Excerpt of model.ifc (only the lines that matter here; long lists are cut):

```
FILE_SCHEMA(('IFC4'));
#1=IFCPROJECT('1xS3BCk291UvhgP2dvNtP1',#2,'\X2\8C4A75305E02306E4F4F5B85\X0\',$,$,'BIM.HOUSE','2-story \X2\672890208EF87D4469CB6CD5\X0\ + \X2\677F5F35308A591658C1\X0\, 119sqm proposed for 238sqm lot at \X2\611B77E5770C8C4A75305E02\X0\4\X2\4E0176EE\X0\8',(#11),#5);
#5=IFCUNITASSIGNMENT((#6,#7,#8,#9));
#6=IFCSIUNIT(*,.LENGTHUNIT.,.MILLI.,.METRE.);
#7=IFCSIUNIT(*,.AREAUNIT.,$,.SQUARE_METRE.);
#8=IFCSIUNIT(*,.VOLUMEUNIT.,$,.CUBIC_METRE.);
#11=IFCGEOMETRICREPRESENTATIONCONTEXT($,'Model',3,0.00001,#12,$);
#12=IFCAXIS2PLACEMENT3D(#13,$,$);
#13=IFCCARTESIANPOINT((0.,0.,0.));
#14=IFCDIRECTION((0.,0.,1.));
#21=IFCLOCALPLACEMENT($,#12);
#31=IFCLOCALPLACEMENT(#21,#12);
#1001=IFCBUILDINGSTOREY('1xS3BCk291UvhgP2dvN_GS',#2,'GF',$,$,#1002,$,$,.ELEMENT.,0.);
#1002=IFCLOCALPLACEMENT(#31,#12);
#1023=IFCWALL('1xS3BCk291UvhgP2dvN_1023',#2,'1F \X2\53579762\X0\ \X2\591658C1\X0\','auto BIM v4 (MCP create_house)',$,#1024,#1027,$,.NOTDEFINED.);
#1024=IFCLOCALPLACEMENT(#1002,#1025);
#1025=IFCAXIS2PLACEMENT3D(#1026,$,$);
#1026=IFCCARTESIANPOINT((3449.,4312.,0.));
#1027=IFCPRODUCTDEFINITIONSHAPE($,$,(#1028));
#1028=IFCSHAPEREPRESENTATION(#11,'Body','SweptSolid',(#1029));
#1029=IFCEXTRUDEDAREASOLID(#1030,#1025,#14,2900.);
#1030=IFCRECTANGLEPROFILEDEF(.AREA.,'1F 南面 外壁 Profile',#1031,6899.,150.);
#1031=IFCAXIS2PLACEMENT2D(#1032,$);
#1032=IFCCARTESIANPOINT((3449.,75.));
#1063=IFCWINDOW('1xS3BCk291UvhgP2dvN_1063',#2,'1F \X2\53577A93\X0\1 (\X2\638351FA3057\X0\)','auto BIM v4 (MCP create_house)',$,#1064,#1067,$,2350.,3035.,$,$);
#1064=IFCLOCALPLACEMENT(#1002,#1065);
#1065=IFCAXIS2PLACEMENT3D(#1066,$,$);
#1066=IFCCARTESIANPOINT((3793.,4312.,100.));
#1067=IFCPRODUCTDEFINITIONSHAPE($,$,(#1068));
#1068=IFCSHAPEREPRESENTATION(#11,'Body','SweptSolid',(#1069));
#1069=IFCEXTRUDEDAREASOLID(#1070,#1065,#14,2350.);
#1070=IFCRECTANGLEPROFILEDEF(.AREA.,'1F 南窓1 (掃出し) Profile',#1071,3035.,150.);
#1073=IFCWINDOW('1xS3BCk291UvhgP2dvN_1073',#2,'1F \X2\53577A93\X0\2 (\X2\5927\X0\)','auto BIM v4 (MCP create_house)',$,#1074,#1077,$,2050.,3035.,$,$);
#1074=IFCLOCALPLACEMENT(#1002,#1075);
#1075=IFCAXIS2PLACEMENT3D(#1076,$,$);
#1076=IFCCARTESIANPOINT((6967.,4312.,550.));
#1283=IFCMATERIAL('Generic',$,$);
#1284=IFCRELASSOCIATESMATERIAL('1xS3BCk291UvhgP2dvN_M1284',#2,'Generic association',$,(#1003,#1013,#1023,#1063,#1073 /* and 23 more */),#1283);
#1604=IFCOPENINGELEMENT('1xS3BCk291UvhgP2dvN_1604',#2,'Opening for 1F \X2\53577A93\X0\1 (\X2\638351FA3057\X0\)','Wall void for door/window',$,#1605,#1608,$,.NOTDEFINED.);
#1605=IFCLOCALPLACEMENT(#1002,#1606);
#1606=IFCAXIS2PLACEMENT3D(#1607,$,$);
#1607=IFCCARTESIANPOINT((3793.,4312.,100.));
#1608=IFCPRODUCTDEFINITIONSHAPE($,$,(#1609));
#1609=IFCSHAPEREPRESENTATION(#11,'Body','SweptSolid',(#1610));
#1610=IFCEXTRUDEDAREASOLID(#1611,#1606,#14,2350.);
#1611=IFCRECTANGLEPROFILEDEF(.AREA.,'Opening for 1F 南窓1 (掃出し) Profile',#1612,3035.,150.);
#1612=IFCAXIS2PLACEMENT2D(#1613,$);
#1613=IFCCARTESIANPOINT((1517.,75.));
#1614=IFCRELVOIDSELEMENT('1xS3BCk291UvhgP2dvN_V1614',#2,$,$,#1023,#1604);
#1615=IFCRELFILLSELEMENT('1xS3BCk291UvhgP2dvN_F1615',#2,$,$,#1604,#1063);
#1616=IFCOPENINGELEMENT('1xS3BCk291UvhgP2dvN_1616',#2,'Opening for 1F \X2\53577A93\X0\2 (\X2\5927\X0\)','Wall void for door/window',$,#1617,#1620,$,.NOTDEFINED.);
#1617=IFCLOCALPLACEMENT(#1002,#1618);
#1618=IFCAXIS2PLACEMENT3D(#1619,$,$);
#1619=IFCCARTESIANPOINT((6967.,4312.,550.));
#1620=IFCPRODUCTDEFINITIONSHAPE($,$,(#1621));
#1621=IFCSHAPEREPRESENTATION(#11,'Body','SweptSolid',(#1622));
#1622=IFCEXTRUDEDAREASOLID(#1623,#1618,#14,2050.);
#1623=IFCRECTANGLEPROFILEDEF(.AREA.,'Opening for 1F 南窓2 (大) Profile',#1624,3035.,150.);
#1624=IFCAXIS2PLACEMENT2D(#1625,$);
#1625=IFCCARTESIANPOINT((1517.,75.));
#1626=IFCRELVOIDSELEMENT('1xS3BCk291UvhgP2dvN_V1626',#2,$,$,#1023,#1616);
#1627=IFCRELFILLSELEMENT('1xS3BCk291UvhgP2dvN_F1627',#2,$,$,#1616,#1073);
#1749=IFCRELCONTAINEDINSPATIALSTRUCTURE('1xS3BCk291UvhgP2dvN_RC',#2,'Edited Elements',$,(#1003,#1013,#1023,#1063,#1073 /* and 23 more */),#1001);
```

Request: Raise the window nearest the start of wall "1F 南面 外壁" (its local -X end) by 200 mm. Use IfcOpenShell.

```python
import numpy as np
import ifcopenshell
import ifcopenshell.api.geometry
import ifcopenshell.util.placement
import ifcopenshell.util.unit

model = ifcopenshell.open("model.ifc")
unit_scale = ifcopenshell.util.unit.calculate_unit_scale(model)

window = model.by_guid("1xS3BCk291UvhgP2dvN_1063")
opening = window.FillsVoids[0].RelatingOpeningElement
dz = 200.0

shift = np.array([0.0, 0.0, dz])
# The window is not placed relative to its opening, so move both.
for product in (opening, window):
    matrix = ifcopenshell.util.placement.get_local_placement(product.ObjectPlacement)
    matrix[:3, 3] += shift
    ifcopenshell.api.geometry.edit_object_placement(model, product=product, matrix=matrix, is_si=False)

print(f"moved by {dz * unit_scale:+.3f} m")

model.write("model_updated.ifc")
```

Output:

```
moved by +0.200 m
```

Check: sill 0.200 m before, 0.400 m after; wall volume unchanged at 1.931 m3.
